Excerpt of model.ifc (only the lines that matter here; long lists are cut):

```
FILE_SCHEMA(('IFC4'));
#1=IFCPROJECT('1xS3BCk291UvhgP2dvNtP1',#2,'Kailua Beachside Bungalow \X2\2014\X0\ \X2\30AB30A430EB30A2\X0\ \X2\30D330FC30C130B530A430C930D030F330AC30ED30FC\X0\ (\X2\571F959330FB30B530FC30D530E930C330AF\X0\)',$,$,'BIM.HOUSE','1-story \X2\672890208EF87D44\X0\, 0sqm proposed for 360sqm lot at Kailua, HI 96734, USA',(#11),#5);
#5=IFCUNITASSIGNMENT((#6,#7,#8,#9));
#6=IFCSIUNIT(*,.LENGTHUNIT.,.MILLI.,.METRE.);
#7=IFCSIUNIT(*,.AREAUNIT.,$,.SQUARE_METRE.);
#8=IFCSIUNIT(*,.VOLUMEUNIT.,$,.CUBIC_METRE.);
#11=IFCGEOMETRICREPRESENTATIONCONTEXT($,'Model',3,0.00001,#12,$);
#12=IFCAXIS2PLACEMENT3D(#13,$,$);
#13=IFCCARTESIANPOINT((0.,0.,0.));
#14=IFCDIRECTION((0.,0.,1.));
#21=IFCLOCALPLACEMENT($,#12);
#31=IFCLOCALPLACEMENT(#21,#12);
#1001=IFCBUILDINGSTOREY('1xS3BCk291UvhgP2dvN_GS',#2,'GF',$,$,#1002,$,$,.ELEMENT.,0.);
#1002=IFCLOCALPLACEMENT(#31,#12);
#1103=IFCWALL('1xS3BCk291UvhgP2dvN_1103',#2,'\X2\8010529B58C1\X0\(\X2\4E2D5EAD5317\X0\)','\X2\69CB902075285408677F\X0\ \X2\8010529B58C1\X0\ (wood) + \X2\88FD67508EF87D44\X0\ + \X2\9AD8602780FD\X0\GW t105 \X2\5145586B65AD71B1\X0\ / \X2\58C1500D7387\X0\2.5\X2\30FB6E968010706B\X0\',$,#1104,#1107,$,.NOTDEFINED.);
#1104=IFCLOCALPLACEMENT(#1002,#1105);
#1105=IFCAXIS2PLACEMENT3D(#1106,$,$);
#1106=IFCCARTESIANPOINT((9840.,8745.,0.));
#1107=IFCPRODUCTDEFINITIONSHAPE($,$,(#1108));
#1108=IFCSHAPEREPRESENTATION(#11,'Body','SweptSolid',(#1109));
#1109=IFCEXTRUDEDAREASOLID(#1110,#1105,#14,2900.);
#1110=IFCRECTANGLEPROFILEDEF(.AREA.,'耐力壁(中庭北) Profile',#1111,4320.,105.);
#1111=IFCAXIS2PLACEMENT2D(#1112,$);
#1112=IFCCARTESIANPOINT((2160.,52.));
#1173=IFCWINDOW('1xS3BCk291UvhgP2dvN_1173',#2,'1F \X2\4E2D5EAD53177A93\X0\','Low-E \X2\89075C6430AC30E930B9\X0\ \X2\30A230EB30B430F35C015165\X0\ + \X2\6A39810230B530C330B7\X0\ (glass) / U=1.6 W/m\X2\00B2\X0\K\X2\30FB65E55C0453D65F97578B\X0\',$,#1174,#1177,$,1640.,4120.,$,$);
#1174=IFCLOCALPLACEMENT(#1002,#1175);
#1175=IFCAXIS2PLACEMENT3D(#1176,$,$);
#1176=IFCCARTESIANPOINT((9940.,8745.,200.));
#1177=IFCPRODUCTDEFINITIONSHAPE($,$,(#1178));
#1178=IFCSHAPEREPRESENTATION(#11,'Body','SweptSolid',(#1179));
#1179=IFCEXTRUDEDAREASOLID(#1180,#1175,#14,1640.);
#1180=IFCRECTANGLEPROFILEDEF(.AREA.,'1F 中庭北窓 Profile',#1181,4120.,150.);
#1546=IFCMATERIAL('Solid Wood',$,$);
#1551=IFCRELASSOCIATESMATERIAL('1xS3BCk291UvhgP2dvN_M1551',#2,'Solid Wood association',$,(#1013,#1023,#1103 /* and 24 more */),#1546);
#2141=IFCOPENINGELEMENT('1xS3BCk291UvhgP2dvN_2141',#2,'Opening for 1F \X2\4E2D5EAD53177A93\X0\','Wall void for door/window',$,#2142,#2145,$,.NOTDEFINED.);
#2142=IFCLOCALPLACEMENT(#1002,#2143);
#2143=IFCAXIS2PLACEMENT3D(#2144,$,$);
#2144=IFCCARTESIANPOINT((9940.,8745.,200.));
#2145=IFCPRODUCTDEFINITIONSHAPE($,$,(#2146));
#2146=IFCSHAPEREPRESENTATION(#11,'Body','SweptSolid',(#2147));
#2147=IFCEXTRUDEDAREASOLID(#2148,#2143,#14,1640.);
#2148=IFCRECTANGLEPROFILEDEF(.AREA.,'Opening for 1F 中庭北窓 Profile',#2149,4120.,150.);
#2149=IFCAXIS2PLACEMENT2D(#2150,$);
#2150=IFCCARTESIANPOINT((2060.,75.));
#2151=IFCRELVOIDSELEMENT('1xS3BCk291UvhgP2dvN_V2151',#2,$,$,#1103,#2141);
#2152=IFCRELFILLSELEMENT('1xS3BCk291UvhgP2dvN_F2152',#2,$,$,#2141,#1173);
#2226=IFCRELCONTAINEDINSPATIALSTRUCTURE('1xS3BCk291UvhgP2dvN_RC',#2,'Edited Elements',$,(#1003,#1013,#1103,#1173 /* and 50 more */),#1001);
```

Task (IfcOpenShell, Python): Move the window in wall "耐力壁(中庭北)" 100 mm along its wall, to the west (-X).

```python
import ifcopenshell
import ifcopenshell.api.geometry
import ifcopenshell.util.placement

model = ifcopenshell.open("model.ifc")

window = model.by_guid("1xS3BCk291UvhgP2dvN_1173")
opening = window.FillsVoids[0].RelatingOpeningElement
wall = opening.VoidsElements[0].RelatingBuildingElement

wall_matrix = ifcopenshell.util.placement.get_local_placement(wall.ObjectPlacement)
shift = wall_matrix[:3, 0] * -100.0
before = ifcopenshell.util.placement.get_local_placement(window.ObjectPlacement)[:3, 3].copy()

# The window is not placed relative to its opening, so move both.
for product in (opening, window):
    matrix = ifcopenshell.util.placement.get_local_placement(product.ObjectPlacement)
    matrix[:3, 3] += shift
    ifcopenshell.api.geometry.edit_object_placement(model, product=product, matrix=matrix, is_si=False)

after = ifcopenshell.util.placement.get_local_placement(window.ObjectPlacement)[:3, 3]
print("window moved by", (after - before).round(3) + 0.0)

model.write("model_updated.ifc")
```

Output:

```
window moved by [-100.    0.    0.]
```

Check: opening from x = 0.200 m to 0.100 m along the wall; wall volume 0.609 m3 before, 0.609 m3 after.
